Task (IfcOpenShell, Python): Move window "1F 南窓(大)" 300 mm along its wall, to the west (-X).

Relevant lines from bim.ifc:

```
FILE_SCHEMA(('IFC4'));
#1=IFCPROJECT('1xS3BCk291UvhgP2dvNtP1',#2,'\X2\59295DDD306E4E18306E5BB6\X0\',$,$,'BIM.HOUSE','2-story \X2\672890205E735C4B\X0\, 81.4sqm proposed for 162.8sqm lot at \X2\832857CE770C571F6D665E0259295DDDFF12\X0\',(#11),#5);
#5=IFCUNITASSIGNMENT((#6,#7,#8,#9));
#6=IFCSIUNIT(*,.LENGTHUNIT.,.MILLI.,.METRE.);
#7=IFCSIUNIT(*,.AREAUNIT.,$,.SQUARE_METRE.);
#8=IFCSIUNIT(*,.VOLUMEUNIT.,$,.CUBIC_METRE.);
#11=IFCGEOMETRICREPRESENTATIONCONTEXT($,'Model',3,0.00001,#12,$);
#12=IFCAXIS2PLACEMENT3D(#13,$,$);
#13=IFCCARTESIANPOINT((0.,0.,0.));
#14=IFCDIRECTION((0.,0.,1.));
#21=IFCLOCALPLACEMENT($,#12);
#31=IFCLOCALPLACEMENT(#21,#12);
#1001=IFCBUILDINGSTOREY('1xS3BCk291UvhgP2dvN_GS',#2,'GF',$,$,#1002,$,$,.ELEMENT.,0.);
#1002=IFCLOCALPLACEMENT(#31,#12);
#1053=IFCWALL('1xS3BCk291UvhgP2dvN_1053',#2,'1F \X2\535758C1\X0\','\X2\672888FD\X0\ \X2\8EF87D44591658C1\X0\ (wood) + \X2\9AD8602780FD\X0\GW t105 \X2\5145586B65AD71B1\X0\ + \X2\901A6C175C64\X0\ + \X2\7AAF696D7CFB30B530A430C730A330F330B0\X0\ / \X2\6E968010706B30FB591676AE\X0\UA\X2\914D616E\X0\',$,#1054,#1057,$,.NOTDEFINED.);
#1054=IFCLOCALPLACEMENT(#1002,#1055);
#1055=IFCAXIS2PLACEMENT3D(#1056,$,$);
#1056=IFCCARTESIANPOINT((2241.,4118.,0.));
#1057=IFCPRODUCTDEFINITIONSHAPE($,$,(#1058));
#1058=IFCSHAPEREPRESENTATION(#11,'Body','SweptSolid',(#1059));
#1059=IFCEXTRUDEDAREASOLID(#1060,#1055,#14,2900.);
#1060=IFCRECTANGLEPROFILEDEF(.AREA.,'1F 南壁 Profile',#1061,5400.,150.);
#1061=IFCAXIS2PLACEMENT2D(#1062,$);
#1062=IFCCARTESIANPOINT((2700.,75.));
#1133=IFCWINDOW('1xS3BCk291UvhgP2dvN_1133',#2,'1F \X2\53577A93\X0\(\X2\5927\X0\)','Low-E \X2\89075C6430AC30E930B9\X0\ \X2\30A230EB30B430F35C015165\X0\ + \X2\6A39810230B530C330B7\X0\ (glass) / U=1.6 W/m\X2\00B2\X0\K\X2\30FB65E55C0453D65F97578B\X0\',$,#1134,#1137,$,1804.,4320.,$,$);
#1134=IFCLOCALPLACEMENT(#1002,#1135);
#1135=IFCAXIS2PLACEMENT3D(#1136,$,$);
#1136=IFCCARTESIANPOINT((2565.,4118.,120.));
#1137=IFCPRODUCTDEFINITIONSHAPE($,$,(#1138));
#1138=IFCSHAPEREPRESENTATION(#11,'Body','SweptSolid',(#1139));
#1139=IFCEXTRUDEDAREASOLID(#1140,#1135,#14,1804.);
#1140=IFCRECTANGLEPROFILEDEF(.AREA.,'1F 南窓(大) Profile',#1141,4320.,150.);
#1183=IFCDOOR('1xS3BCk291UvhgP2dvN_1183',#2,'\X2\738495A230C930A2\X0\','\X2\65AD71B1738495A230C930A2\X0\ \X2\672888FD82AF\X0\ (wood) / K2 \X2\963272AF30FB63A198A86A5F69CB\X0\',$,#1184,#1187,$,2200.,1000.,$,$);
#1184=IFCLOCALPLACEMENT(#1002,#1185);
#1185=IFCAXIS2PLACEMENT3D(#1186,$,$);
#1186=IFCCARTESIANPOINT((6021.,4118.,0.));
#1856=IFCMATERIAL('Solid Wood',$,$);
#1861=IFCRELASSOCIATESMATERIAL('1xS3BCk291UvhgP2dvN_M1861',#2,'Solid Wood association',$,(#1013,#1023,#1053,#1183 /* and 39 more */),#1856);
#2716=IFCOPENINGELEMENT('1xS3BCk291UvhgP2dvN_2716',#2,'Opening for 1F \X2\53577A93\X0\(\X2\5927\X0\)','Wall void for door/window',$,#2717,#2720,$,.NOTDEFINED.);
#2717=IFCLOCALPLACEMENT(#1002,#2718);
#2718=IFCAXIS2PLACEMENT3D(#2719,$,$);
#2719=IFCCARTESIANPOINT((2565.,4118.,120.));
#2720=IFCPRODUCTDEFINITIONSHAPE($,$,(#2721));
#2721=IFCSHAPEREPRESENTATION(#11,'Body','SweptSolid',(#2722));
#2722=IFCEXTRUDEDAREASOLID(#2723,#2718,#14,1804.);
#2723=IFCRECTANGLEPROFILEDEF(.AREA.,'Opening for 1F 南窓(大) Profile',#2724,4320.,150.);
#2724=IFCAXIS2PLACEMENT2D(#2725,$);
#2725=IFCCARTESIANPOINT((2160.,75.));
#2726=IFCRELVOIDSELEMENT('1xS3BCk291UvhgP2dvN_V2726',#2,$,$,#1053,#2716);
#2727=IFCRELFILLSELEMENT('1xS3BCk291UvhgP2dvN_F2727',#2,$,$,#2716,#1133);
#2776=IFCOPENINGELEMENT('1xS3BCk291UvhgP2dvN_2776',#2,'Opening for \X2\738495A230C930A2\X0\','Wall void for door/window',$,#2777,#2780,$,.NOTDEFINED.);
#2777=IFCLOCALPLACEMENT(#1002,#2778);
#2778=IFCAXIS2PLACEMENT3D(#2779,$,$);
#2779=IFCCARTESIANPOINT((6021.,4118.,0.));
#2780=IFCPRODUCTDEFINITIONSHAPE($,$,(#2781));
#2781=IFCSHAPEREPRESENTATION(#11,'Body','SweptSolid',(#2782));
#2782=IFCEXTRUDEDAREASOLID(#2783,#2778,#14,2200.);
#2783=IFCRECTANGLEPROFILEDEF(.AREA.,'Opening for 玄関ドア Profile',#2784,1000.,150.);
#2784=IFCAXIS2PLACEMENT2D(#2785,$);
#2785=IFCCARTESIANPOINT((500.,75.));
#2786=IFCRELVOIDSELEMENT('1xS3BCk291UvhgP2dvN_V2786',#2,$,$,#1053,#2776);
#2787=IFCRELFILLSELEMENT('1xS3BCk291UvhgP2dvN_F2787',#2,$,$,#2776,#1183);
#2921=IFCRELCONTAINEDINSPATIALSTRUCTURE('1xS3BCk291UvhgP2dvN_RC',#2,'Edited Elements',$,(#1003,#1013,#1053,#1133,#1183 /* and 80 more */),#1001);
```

```python
import ifcopenshell
import ifcopenshell.api.geometry
import ifcopenshell.util.placement

model = ifcopenshell.open("bim.ifc")

window = model.by_guid("1xS3BCk291UvhgP2dvN_1133")
opening = window.FillsVoids[0].RelatingOpeningElement
wall = opening.VoidsElements[0].RelatingBuildingElement

wall_matrix = ifcopenshell.util.placement.get_local_placement(wall.ObjectPlacement)
shift = wall_matrix[:3, 0] * -300.0
before = ifcopenshell.util.placement.get_local_placement(window.ObjectPlacement)[:3, 3].copy()

# The window is not placed relative to its opening, so move both.
for product in (opening, window):
    matrix = ifcopenshell.util.placement.get_local_placement(product.ObjectPlacement)
    matrix[:3, 3] += shift
    ifcopenshell.api.geometry.edit_object_placement(model, product=product, matrix=matrix, is_si=False)

after = ifcopenshell.util.placement.get_local_placement(window.ObjectPlacement)[:3, 3]
print("window moved by", (after - before).round(3) + 0.0)

model.write("bim_edited.ifc")
```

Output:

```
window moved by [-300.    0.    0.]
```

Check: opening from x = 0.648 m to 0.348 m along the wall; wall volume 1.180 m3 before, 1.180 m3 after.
